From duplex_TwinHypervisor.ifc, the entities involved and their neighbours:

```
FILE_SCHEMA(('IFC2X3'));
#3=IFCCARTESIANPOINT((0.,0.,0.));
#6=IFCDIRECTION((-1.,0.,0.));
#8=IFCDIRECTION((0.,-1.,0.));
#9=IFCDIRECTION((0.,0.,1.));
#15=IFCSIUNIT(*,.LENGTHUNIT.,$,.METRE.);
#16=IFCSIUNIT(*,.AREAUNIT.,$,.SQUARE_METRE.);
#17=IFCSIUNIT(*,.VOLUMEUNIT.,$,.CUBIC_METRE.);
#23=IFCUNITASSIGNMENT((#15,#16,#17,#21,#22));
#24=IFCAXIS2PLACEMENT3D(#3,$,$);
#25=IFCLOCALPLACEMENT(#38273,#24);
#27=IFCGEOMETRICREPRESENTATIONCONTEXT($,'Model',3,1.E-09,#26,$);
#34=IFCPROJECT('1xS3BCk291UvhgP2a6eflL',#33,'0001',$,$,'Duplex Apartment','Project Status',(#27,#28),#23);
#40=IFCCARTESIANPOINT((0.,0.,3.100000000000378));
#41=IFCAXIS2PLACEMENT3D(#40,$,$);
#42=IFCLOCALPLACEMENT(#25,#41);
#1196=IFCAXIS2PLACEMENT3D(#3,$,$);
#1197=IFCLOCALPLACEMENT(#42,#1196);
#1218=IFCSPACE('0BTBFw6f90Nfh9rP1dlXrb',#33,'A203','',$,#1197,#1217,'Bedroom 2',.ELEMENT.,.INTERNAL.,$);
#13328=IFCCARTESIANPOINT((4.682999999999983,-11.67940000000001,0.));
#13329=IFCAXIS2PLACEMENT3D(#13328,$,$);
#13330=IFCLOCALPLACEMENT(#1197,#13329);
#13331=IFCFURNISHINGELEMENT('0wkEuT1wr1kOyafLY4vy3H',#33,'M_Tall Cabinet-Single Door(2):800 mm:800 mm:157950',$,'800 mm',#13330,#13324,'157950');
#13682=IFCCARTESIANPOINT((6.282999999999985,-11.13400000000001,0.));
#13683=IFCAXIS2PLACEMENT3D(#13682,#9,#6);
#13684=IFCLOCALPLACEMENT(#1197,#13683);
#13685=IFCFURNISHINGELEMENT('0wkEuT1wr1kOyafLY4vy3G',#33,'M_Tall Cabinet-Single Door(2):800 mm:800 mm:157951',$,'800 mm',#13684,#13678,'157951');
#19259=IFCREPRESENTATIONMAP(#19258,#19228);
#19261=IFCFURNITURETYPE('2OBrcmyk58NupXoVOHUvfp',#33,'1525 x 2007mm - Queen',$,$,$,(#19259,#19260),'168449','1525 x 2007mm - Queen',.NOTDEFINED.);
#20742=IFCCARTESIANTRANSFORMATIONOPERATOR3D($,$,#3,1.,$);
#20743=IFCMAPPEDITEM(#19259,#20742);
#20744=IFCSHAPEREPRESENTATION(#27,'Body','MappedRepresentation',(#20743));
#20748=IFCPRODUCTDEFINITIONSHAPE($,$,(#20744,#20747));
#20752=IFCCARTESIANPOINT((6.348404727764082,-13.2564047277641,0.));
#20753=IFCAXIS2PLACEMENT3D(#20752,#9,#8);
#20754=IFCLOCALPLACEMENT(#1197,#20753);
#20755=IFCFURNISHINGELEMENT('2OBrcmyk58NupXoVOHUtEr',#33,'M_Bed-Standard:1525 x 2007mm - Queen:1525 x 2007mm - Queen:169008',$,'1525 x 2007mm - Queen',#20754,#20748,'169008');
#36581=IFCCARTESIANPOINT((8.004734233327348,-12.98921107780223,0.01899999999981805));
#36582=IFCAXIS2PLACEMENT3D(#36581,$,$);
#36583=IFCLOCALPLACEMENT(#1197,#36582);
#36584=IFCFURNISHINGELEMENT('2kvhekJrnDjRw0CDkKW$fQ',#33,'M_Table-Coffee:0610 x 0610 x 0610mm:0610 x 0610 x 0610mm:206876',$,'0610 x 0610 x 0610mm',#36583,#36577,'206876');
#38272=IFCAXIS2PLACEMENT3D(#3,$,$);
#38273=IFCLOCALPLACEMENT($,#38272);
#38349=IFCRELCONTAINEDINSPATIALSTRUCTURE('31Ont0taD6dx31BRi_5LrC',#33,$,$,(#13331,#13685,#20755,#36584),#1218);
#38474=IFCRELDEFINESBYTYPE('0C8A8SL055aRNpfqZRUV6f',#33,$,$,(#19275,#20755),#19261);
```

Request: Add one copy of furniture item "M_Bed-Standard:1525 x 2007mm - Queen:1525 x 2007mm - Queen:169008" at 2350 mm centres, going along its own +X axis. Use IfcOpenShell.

```python
import ifcopenshell
import ifcopenshell.api.geometry
import ifcopenshell.api.root
import ifcopenshell.util.element
import ifcopenshell.util.placement
import ifcopenshell.util.unit

model = ifcopenshell.open("duplex_TwinHypervisor.ifc")
unit_scale = ifcopenshell.util.unit.calculate_unit_scale(model)


def reuse_history(source, copy):
    """copy_class also copies each property set's owner history, people and application; keep the originals."""
    for rel in copy.IsDefinedBy:
        if rel.is_a("IfcRelDefinesByProperties") and (history := rel.RelatingPropertyDefinition.OwnerHistory):
            rel.RelatingPropertyDefinition.OwnerHistory = source.OwnerHistory
            ifcopenshell.util.element.remove_deep2(model, history)


source = model.by_guid("2OBrcmyk58NupXoVOHUtEr")
base = ifcopenshell.util.placement.get_local_placement(source.ObjectPlacement)
step = base[:3, 0] * 2.35 / unit_scale

for i in range(1, 2):
    copy = ifcopenshell.api.root.copy_class(model, product=source)
    copy.Representation = ifcopenshell.util.element.copy_deep(
        model, source.Representation, exclude=["IfcGeometricRepresentationContext", "IfcRepresentationMap"]
    )
    copy.Name = "M_Bed-Standard:1525 x 2007mm - Queen:1525 x 2007mm - Queen"
    copy.Tag = None
    reuse_history(source, copy)
    matrix = base.copy()
    matrix[:3, 3] += i * step
    print("added at", matrix[:3, 3].round(3) + 0.0)
    ifcopenshell.api.geometry.edit_object_placement(model, product=copy, matrix=matrix, is_si=False)

model.write("duplex_TwinHypervisor-out.ifc")
```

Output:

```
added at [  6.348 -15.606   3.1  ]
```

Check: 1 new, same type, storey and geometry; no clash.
